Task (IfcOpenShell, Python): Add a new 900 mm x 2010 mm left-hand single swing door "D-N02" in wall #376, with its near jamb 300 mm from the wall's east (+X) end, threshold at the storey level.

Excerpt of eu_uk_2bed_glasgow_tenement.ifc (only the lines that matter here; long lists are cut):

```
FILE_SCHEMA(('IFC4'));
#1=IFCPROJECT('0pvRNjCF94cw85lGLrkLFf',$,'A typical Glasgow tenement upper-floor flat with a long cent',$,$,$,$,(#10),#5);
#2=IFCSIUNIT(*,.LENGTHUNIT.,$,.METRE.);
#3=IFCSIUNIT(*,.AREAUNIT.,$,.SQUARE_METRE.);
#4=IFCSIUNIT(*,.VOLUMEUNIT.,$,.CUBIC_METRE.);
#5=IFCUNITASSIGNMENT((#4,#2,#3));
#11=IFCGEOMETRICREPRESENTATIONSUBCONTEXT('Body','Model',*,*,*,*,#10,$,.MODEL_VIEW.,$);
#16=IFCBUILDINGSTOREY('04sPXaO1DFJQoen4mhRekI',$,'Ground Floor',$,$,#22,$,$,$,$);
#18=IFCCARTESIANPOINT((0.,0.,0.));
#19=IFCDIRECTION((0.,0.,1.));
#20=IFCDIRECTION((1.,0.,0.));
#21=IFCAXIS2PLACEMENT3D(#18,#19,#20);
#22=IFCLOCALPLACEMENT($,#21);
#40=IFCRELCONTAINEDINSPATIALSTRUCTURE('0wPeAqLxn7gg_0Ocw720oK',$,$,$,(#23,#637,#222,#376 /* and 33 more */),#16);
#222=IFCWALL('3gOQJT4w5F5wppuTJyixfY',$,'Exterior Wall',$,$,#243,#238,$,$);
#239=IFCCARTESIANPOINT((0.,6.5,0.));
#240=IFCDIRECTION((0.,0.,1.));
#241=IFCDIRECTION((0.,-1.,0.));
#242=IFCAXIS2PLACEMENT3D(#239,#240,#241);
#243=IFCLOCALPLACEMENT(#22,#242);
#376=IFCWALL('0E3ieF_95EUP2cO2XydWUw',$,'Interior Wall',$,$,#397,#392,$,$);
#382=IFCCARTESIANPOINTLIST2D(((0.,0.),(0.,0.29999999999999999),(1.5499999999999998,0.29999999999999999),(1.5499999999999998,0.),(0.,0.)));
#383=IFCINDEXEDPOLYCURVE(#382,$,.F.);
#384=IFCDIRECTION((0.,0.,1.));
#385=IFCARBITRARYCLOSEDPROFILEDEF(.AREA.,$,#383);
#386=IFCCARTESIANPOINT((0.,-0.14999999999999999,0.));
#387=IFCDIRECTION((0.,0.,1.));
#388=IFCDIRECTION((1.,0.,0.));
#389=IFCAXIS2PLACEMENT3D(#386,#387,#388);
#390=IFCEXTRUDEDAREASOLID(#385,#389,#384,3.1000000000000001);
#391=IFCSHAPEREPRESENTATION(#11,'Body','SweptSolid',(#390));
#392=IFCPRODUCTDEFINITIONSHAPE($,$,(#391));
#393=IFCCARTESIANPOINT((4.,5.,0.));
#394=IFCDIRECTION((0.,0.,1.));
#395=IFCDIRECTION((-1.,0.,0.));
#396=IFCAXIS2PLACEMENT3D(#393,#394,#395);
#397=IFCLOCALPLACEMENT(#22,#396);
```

```python
import numpy as np
import ifcopenshell
import ifcopenshell.api.feature
import ifcopenshell.api.geometry
import ifcopenshell.api.root
import ifcopenshell.api.spatial
import ifcopenshell.geom
import ifcopenshell.util.element
import ifcopenshell.util.placement
import ifcopenshell.util.representation
import ifcopenshell.util.shape
import ifcopenshell.util.unit

model = ifcopenshell.open("eu_uk_2bed_glasgow_tenement.ifc")
unit_scale = ifcopenshell.util.unit.calculate_unit_scale(model)
settings = ifcopenshell.geom.settings()


def volume(element):
    """Net volume in cubic metres, openings subtracted."""
    shape = ifcopenshell.geom.create_shape(settings, element)
    return ifcopenshell.util.shape.get_volume(shape.geometry)


wall = model.by_guid("0E3ieF_95EUP2cO2XydWUw")
storey = ifcopenshell.util.element.get_container(wall, ifc_class="IfcBuildingStorey")
context = ifcopenshell.util.representation.get_context(model, "Model", "Body", "MODEL_VIEW")
before = volume(wall)

width, height, from_end, sill = 0.9, 2.01, 0.3, 0.0  # metres

# The wall runs along its own X axis, and the end named is its -X end.
wall_shape = ifcopenshell.geom.create_shape(settings, wall)
x, y, z = ifcopenshell.util.shape.get_vertices(wall_shape.geometry).T
start = x.min() + from_end
face, thickness = float(y.min()), float(y.max() - y.min())
wall_matrix = ifcopenshell.util.placement.get_local_placement(wall.ObjectPlacement)
level = ifcopenshell.util.placement.get_local_placement(storey.ObjectPlacement)[2, 3]


def in_wall(x, y):
    """Placement at x, y metres in the wall's axes, at sill height."""
    matrix = wall_matrix.copy()
    matrix[:, 3] = wall_matrix @ np.array([x / unit_scale, y / unit_scale, 0.0, 1.0])
    matrix[2, 3] = level + sill / unit_scale
    return matrix


# Opening: a box that overshoots both wall faces by 50 mm.
opening = ifcopenshell.api.root.create_entity(model, ifc_class="IfcOpeningElement", predefined_type="OPENING")
box = ifcopenshell.api.geometry.add_wall_representation(
    model, context=context, length=width, height=height, thickness=thickness + 0.1
)
ifcopenshell.api.geometry.assign_representation(model, product=opening, representation=box)
ifcopenshell.api.geometry.edit_object_placement(model, product=opening, matrix=in_wall(start, face - 0.05), is_si=False)
ifcopenshell.api.feature.add_feature(model, feature=opening, element=wall)

door = ifcopenshell.api.root.create_entity(model, ifc_class="IfcDoor", name="D-N02", predefined_type="DOOR")
door.OverallWidth, door.OverallHeight = width / unit_scale, height / unit_scale
door.OperationType = "SINGLE_SWING_LEFT"
body = ifcopenshell.api.geometry.add_door_representation(
    model,
    context=context,
    overall_width=door.OverallWidth,
    overall_height=door.OverallHeight,
    operation_type="SINGLE_SWING_LEFT",
    lining_properties={"LiningDepth": thickness / unit_scale, "ThresholdDepth": thickness / unit_scale},
)
ifcopenshell.api.geometry.assign_representation(model, product=door, representation=body)
ifcopenshell.api.spatial.assign_container(model, products=[door], relating_structure=storey)
ifcopenshell.api.feature.add_filling(model, opening=opening, element=door)

# The lining spans the wall, so the door starts at the wall face.
ifcopenshell.api.geometry.edit_object_placement(model, product=door, matrix=in_wall(start, face), is_si=False)

after = volume(wall)

print(f"wall volume {before:.3f} -> {after:.3f} m3")

model.write("eu_uk_2bed_glasgow_tenement_updated.ifc")
```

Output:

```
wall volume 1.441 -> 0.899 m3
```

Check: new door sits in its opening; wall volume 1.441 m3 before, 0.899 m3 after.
